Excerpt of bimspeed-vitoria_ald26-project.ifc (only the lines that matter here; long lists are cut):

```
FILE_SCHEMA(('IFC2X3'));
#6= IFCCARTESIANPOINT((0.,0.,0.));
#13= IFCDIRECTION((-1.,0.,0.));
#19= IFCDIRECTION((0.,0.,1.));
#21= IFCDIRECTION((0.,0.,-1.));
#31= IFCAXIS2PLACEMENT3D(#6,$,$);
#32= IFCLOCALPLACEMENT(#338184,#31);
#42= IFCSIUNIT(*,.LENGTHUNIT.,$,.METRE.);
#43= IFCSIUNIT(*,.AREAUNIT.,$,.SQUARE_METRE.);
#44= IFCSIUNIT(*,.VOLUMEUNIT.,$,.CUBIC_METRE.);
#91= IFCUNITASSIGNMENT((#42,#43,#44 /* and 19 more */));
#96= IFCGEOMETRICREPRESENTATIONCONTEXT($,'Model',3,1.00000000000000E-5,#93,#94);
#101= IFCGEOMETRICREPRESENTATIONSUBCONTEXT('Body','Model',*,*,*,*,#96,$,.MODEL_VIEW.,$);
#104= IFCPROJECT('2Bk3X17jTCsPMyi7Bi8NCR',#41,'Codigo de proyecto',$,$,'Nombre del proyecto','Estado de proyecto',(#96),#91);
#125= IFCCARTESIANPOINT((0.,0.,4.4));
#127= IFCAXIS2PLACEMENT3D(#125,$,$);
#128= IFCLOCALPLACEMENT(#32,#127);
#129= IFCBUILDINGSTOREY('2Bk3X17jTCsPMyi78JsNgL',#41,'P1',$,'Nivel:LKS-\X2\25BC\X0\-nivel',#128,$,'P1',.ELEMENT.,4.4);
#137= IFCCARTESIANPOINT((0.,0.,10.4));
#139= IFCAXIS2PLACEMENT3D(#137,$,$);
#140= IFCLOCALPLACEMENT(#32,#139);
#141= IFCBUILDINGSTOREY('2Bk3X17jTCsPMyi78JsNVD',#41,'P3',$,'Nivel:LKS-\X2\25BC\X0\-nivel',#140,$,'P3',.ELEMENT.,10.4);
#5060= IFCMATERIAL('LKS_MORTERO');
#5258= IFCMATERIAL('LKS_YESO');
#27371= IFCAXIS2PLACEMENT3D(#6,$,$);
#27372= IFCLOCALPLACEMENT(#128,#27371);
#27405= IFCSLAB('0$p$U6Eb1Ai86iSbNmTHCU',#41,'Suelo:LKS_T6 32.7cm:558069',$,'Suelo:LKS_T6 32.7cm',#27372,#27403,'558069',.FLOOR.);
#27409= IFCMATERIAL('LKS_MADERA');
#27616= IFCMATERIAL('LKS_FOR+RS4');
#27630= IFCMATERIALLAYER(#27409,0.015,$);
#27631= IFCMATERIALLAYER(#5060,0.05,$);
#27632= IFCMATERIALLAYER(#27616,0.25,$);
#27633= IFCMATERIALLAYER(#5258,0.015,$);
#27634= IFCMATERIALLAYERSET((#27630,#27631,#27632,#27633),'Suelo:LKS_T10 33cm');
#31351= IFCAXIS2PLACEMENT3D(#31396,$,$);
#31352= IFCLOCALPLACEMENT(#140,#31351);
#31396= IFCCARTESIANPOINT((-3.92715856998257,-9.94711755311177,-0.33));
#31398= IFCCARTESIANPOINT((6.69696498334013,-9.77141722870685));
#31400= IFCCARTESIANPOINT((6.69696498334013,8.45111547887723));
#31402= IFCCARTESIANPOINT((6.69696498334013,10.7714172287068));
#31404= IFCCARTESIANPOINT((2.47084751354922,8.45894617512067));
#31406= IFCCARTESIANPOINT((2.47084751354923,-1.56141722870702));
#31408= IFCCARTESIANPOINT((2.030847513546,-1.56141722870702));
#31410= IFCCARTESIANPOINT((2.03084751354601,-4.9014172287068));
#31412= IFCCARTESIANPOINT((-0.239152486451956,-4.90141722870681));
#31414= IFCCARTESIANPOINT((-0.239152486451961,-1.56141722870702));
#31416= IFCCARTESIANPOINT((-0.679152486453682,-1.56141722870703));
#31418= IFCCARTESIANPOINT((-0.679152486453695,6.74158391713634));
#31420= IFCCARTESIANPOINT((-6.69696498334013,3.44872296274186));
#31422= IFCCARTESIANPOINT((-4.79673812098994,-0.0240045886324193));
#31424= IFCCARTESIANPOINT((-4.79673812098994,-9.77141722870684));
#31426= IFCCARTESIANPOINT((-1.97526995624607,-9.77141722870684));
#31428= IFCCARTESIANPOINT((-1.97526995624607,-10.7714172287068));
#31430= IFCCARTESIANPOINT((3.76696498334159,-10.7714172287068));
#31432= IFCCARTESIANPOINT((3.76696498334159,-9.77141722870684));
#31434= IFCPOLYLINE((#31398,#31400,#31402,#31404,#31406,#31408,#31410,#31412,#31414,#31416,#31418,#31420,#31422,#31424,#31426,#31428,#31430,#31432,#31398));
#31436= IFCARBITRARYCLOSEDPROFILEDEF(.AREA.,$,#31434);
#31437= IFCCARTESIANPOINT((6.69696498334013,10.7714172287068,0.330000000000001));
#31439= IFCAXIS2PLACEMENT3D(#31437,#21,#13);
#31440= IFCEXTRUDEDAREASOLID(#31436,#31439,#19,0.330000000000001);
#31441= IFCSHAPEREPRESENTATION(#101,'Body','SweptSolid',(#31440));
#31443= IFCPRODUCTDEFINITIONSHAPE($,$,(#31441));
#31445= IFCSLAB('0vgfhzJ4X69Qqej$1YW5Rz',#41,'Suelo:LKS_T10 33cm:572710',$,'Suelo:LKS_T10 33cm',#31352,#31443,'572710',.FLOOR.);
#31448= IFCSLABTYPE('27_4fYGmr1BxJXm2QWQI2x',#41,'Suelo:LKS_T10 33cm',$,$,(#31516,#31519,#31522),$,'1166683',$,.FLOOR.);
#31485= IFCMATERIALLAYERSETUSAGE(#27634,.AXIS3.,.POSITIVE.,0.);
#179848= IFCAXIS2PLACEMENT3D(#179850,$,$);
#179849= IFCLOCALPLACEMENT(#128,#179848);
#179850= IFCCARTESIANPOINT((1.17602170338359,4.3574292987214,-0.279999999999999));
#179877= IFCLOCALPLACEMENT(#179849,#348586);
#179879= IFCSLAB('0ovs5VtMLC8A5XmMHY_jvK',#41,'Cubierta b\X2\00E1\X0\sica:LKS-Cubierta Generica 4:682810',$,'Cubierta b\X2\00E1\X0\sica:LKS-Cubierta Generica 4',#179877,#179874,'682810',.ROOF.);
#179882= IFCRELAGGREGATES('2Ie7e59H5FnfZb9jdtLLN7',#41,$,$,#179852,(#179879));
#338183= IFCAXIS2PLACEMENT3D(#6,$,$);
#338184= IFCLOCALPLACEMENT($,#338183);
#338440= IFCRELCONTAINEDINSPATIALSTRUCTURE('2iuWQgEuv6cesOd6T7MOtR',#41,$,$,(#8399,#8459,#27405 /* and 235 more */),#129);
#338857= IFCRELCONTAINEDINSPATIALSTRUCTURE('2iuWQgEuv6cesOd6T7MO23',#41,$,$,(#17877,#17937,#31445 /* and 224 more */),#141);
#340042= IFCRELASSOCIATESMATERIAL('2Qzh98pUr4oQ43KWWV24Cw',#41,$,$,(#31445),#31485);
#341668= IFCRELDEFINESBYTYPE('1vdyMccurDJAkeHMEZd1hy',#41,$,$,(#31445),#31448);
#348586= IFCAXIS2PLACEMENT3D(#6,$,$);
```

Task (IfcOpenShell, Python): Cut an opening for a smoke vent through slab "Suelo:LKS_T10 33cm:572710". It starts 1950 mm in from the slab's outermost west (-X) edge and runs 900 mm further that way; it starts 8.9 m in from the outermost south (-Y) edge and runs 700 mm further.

```python
import numpy as np
import ifcopenshell
import ifcopenshell.api.feature
import ifcopenshell.api.geometry
import ifcopenshell.api.root
import ifcopenshell.geom
import ifcopenshell.util.placement
import ifcopenshell.util.representation
import ifcopenshell.util.shape
import ifcopenshell.util.unit

model = ifcopenshell.open("bimspeed-vitoria_ald26-project.ifc")
unit_scale = ifcopenshell.util.unit.calculate_unit_scale(model)
settings = ifcopenshell.geom.settings()


def volume(element):
    """Net volume in cubic metres, openings subtracted."""
    shape = ifcopenshell.geom.create_shape(settings, element)
    return ifcopenshell.util.shape.get_volume(shape.geometry)


slab = model.by_guid("0vgfhzJ4X69Qqej$1YW5Rz")
before = volume(slab)

# Extent in the slab's own axes, in metres. The edges named are its -X and -Y sides.
slab_shape = ifcopenshell.geom.create_shape(settings, slab)
vertices = ifcopenshell.util.shape.get_vertices(slab_shape.geometry)
x_min, y_min, bottom = vertices.min(axis=0)
top = vertices[:, 2].max()

opening = ifcopenshell.api.root.create_entity(model, ifc_class="IfcOpeningElement", name="Smoke vent opening")
context = ifcopenshell.util.representation.get_context(model, "Model", "Body", "MODEL_VIEW")
width, depth = 0.9, 0.7
outline = [(0.0, 0.0), (width, 0.0), (width, depth), (0.0, depth), (0.0, 0.0)]
# Overshoot both faces by 50 mm so the cut is clean.
shape = ifcopenshell.api.geometry.add_slab_representation(
    model, context=context, depth=top - bottom + 0.1, polyline=outline
)
ifcopenshell.api.geometry.assign_representation(model, product=opening, representation=shape)

matrix = ifcopenshell.util.placement.get_local_placement(slab.ObjectPlacement)
matrix[:, 3] = matrix @ np.append(np.array([x_min + 1.95, y_min + 8.9, bottom - 0.05]) / unit_scale, 1.0)
ifcopenshell.api.geometry.edit_object_placement(model, product=opening, matrix=matrix, is_si=False)
ifcopenshell.api.feature.add_feature(model, feature=opening, element=slab)

after = volume(slab)

print(f"slab volume {before:.3f} -> {after:.3f} m3")

model.write("bimspeed-vitoria_ald26-project_updated.ifc")
```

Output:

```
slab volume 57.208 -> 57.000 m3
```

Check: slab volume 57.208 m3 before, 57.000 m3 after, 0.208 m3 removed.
